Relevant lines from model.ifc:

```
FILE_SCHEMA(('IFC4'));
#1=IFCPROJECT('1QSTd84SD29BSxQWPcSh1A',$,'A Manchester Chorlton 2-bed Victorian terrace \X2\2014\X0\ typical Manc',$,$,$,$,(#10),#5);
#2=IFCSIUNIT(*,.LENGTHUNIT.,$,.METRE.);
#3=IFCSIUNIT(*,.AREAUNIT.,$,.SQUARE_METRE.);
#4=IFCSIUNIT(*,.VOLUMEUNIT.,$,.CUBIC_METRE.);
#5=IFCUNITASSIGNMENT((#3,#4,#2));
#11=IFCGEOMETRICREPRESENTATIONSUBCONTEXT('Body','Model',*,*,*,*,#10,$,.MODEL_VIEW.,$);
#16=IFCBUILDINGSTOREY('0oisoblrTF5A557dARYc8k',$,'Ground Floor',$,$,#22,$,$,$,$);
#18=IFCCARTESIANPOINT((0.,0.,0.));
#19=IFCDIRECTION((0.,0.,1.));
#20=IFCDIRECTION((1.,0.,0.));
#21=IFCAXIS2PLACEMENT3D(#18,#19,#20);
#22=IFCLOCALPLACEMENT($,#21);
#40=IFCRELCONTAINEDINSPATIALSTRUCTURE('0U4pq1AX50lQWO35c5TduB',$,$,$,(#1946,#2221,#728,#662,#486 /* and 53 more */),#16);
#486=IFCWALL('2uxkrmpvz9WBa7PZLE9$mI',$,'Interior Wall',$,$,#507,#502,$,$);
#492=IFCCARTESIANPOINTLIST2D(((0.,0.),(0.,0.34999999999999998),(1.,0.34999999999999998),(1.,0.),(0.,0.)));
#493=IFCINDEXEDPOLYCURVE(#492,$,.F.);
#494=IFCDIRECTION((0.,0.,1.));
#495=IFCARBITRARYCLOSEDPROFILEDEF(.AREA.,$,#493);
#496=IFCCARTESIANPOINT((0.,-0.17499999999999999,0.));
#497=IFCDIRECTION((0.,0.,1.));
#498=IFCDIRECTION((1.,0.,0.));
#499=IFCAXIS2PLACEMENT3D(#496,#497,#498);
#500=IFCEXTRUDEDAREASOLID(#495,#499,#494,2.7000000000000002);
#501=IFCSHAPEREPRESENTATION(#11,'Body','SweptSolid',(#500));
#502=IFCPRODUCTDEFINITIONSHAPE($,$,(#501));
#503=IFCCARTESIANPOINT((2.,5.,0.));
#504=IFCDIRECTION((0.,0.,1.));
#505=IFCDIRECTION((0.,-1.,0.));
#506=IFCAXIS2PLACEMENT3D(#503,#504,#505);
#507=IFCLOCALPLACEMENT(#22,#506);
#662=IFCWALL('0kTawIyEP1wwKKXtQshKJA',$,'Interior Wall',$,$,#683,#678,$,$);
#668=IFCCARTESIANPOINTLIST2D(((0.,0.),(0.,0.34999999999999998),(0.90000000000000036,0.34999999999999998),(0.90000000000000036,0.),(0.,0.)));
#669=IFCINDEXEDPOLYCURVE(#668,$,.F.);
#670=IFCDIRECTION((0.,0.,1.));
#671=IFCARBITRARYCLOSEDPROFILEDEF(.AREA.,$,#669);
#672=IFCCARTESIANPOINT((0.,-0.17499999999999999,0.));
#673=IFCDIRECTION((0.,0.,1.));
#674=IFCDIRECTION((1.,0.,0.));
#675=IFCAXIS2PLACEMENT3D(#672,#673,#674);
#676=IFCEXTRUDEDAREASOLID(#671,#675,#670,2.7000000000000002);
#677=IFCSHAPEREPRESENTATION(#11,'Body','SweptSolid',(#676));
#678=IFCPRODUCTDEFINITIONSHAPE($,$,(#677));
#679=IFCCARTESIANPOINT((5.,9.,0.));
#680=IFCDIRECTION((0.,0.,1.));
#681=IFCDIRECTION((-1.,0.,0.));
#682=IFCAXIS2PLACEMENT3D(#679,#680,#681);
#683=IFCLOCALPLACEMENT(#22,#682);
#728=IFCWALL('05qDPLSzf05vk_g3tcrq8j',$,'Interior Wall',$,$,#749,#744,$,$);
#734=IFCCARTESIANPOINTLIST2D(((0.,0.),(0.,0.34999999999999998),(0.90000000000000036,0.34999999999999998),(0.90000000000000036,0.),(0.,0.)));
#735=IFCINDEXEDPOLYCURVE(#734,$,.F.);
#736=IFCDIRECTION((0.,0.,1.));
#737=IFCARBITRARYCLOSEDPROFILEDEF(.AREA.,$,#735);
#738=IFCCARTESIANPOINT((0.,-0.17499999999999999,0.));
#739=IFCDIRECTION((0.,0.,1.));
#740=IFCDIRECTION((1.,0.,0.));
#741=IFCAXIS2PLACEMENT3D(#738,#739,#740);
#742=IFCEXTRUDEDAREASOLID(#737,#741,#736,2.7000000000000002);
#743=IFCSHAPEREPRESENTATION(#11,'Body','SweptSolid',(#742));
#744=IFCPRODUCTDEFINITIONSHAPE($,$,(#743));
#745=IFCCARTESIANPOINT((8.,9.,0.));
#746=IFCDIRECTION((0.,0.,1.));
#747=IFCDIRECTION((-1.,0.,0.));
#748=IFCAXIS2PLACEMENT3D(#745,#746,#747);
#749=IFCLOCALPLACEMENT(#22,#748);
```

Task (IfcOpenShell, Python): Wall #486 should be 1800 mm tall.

```python
import ifcopenshell
import ifcopenshell.geom
import ifcopenshell.util.representation
import ifcopenshell.util.shape
import ifcopenshell.util.unit

model = ifcopenshell.open("model.ifc")
unit_scale = ifcopenshell.util.unit.calculate_unit_scale(model)
settings = ifcopenshell.geom.settings()


def volume(element):
    """Net volume in cubic metres, openings subtracted."""
    shape = ifcopenshell.geom.create_shape(settings, element)
    return ifcopenshell.util.shape.get_volume(shape.geometry)


wall = model.by_guid("2uxkrmpvz9WBa7PZLE9$mI")
before = volume(wall)

body = ifcopenshell.util.representation.get_representation(wall, "Model", "Body")
solid = body.Items[0]
old_height = solid.Depth
solid.Depth = 1.8 / unit_scale
after = volume(wall)

print(f"height {old_height:g} -> {solid.Depth:g}, volume {before:.3f} -> {after:.3f} m3")

model.write("model-out.ifc")
```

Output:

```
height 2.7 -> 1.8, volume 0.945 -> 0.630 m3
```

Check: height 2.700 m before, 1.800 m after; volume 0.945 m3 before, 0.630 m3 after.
